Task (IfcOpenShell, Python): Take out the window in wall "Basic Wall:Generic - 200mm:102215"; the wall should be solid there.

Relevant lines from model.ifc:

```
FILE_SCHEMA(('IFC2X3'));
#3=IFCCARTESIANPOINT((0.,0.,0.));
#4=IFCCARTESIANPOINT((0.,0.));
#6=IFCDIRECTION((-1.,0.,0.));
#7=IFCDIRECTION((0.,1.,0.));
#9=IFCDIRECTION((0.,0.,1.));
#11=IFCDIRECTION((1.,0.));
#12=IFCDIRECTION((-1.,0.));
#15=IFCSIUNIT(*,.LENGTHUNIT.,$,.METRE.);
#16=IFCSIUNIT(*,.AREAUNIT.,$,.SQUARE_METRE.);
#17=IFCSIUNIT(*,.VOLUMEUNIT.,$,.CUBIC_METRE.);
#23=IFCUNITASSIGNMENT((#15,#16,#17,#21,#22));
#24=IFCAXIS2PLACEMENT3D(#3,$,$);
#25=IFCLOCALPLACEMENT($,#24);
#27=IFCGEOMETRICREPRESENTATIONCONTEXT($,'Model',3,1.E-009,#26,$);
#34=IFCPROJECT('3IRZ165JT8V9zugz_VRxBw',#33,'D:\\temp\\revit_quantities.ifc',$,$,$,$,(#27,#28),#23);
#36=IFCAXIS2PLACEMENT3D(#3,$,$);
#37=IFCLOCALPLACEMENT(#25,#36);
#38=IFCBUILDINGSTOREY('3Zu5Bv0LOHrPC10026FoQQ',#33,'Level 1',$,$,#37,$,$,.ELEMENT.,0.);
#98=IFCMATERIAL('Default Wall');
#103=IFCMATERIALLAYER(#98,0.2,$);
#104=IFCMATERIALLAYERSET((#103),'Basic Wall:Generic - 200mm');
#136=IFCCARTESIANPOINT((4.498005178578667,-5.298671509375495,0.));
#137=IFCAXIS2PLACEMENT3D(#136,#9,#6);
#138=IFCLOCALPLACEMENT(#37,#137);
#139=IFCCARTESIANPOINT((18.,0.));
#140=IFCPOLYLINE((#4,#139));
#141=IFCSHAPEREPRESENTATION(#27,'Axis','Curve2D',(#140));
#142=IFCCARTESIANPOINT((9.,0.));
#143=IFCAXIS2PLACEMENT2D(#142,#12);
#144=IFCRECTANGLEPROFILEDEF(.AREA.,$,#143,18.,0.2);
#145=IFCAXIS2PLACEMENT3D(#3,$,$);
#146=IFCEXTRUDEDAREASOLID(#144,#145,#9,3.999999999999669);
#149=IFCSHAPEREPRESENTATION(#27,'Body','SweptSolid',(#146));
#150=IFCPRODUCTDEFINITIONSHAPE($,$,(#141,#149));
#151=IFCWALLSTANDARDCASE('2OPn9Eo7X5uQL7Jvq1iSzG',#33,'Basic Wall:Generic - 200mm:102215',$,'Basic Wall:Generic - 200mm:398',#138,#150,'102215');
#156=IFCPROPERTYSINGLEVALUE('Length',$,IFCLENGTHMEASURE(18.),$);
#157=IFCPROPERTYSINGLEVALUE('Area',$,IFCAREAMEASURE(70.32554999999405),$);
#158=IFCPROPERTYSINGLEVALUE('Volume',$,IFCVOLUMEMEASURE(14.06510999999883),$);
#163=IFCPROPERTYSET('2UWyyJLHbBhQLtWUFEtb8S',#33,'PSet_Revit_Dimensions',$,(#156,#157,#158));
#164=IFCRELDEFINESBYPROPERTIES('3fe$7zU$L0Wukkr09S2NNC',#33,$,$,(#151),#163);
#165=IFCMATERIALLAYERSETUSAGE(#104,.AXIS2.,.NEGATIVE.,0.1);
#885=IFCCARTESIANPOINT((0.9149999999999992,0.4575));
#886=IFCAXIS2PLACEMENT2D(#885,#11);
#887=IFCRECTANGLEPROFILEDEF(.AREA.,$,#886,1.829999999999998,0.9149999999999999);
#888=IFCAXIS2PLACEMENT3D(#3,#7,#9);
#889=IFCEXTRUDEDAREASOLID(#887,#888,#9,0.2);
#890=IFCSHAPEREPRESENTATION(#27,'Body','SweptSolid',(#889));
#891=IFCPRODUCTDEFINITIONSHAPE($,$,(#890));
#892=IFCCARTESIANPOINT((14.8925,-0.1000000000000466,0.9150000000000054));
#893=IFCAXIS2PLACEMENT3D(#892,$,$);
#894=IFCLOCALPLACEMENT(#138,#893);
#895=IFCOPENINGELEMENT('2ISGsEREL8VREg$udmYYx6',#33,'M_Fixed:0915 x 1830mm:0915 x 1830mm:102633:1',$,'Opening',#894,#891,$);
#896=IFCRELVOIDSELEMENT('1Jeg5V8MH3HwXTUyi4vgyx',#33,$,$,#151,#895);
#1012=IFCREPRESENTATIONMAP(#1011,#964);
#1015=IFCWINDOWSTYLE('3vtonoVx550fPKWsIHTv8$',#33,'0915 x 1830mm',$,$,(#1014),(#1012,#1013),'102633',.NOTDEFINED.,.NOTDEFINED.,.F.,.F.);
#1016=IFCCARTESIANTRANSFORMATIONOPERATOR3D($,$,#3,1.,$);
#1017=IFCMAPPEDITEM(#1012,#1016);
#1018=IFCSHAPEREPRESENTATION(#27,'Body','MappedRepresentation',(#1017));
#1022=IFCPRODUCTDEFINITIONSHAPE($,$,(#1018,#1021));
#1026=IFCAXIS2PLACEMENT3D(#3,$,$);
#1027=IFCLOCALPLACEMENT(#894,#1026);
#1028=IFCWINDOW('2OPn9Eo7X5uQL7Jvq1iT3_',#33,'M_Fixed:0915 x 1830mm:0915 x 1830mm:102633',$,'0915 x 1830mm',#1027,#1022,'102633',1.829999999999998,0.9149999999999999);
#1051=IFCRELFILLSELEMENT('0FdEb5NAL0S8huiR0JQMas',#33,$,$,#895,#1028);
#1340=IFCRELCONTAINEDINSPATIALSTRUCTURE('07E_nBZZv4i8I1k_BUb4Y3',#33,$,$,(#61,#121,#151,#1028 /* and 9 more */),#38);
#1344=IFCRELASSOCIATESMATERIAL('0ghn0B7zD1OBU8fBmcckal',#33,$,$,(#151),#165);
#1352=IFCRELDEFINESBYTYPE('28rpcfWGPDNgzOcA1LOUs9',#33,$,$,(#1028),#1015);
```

```python
import ifcopenshell
import ifcopenshell.api.feature
import ifcopenshell.api.pset
import ifcopenshell.api.root
import ifcopenshell.geom
import ifcopenshell.util.element
import ifcopenshell.util.shape
import ifcopenshell.util.unit

model = ifcopenshell.open("model.ifc")
area_scale = ifcopenshell.util.unit.calculate_unit_scale(model, "AREAUNIT")
volume_scale = ifcopenshell.util.unit.calculate_unit_scale(model, "VOLUMEUNIT")
settings = ifcopenshell.geom.settings()


def volume(element):
    """Net volume in cubic metres, openings subtracted."""
    shape = ifcopenshell.geom.create_shape(settings, element)
    return ifcopenshell.util.shape.get_volume(shape.geometry)


window = model.by_id(1028)
opening = window.FillsVoids[0].RelatingOpeningElement
wall = opening.VoidsElements[0].RelatingBuildingElement
before = volume(wall)

ifcopenshell.api.root.remove_product(model, product=window)
ifcopenshell.api.feature.remove_feature(model, feature=opening)

after = volume(wall)
thickness = 0.2  # wall thickness in metres

# Update the wall's stored quantities.
pset = model.by_id(ifcopenshell.util.element.get_pset(wall, "PSet_Revit_Dimensions", should_inherit=False)["id"])
ifcopenshell.api.pset.edit_pset(model, pset=pset, properties={
    "Area": model.create_entity("IfcAreaMeasure", after / thickness / area_scale),
    "Volume": model.create_entity("IfcVolumeMeasure", after / volume_scale),
})

print(f"wall volume {before:.3f} -> {after:.3f} m3")

model.write("model_v2.ifc")
```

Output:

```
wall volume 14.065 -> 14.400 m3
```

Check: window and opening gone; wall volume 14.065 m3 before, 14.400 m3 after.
